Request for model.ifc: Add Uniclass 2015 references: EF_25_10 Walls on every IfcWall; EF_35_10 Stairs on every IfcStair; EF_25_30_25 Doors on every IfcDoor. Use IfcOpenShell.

First a look at what the model holds.

```python
import ifcopenshell

model = ifcopenshell.open("model.ifc")
print(model.schema)
print("classifications:", [c.Name for c in model.by_type("IfcClassification")])
for ifc_class in ("IfcDoor", "IfcRoof", "IfcStair", "IfcWall", "IfcWindow"):
    print(ifc_class, len(model.by_type(ifc_class)))
```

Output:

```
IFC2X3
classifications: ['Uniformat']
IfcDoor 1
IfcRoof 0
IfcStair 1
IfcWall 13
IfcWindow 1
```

```python
import ifcopenshell
import ifcopenshell.api.classification

model = ifcopenshell.open("model.ifc")

# IFC2X3 requires Source and Edition and has no link from the project to the system.
system = model.create_entity("IfcClassification", Source="NBS", Edition="2015", Name="Uniclass 2015")

codes = {
    "IfcWall": ("EF_25_10", "Walls"),
    "IfcStair": ("EF_35_10", "Stairs"),
    "IfcDoor": ("EF_25_30_25", "Doors"),
}
for ifc_class, (code, name) in codes.items():
    products = model.by_type(ifc_class)
    ifcopenshell.api.classification.add_reference(
        model, products=products, classification=system, identification=code, name=name
    )
    print(code, len(products))

model.write("model_v2.ifc")
```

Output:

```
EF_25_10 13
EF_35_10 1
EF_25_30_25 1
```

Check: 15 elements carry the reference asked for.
